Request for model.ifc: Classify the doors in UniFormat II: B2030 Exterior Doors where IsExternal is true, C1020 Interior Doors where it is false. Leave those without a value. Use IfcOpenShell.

First a look at what the model holds.

```python
import ifcopenshell
import ifcopenshell.util.element

model = ifcopenshell.open("model.ifc")
print(model.schema)
print("classifications:", [c.Name for c in model.by_type("IfcClassification")])
values = [ifcopenshell.util.element.get_pset(e, "Pset_DoorCommon", "IsExternal") for e in model.by_type("IfcDoor")]
for value in (True, False, None):
    print("IsExternal", value, values.count(value))
```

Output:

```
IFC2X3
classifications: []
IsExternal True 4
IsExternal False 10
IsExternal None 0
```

```python
import ifcopenshell
import ifcopenshell.api.classification
import ifcopenshell.util.element

model = ifcopenshell.open("model.ifc")

# IFC2X3 requires Source and Edition and has no link from the project to the system.
system = model.create_entity("IfcClassification", Source="ASTM", Edition="E1557", Name="UniFormat II")

doors = model.by_type("IfcDoor")
external = {e: ifcopenshell.util.element.get_pset(e, "Pset_DoorCommon", "IsExternal") for e in doors}
for flag, code, name in ((True, "B2030", "Exterior Doors"), (False, "C1020", "Interior Doors")):
    products = [e for e in doors if external[e] is flag]
    ifcopenshell.api.classification.add_reference(
        model, products=products, classification=system, identification=code, name=name
    )
    print(code, len(products))

model.write("model_v2.ifc")
```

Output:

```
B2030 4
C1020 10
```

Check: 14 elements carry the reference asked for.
